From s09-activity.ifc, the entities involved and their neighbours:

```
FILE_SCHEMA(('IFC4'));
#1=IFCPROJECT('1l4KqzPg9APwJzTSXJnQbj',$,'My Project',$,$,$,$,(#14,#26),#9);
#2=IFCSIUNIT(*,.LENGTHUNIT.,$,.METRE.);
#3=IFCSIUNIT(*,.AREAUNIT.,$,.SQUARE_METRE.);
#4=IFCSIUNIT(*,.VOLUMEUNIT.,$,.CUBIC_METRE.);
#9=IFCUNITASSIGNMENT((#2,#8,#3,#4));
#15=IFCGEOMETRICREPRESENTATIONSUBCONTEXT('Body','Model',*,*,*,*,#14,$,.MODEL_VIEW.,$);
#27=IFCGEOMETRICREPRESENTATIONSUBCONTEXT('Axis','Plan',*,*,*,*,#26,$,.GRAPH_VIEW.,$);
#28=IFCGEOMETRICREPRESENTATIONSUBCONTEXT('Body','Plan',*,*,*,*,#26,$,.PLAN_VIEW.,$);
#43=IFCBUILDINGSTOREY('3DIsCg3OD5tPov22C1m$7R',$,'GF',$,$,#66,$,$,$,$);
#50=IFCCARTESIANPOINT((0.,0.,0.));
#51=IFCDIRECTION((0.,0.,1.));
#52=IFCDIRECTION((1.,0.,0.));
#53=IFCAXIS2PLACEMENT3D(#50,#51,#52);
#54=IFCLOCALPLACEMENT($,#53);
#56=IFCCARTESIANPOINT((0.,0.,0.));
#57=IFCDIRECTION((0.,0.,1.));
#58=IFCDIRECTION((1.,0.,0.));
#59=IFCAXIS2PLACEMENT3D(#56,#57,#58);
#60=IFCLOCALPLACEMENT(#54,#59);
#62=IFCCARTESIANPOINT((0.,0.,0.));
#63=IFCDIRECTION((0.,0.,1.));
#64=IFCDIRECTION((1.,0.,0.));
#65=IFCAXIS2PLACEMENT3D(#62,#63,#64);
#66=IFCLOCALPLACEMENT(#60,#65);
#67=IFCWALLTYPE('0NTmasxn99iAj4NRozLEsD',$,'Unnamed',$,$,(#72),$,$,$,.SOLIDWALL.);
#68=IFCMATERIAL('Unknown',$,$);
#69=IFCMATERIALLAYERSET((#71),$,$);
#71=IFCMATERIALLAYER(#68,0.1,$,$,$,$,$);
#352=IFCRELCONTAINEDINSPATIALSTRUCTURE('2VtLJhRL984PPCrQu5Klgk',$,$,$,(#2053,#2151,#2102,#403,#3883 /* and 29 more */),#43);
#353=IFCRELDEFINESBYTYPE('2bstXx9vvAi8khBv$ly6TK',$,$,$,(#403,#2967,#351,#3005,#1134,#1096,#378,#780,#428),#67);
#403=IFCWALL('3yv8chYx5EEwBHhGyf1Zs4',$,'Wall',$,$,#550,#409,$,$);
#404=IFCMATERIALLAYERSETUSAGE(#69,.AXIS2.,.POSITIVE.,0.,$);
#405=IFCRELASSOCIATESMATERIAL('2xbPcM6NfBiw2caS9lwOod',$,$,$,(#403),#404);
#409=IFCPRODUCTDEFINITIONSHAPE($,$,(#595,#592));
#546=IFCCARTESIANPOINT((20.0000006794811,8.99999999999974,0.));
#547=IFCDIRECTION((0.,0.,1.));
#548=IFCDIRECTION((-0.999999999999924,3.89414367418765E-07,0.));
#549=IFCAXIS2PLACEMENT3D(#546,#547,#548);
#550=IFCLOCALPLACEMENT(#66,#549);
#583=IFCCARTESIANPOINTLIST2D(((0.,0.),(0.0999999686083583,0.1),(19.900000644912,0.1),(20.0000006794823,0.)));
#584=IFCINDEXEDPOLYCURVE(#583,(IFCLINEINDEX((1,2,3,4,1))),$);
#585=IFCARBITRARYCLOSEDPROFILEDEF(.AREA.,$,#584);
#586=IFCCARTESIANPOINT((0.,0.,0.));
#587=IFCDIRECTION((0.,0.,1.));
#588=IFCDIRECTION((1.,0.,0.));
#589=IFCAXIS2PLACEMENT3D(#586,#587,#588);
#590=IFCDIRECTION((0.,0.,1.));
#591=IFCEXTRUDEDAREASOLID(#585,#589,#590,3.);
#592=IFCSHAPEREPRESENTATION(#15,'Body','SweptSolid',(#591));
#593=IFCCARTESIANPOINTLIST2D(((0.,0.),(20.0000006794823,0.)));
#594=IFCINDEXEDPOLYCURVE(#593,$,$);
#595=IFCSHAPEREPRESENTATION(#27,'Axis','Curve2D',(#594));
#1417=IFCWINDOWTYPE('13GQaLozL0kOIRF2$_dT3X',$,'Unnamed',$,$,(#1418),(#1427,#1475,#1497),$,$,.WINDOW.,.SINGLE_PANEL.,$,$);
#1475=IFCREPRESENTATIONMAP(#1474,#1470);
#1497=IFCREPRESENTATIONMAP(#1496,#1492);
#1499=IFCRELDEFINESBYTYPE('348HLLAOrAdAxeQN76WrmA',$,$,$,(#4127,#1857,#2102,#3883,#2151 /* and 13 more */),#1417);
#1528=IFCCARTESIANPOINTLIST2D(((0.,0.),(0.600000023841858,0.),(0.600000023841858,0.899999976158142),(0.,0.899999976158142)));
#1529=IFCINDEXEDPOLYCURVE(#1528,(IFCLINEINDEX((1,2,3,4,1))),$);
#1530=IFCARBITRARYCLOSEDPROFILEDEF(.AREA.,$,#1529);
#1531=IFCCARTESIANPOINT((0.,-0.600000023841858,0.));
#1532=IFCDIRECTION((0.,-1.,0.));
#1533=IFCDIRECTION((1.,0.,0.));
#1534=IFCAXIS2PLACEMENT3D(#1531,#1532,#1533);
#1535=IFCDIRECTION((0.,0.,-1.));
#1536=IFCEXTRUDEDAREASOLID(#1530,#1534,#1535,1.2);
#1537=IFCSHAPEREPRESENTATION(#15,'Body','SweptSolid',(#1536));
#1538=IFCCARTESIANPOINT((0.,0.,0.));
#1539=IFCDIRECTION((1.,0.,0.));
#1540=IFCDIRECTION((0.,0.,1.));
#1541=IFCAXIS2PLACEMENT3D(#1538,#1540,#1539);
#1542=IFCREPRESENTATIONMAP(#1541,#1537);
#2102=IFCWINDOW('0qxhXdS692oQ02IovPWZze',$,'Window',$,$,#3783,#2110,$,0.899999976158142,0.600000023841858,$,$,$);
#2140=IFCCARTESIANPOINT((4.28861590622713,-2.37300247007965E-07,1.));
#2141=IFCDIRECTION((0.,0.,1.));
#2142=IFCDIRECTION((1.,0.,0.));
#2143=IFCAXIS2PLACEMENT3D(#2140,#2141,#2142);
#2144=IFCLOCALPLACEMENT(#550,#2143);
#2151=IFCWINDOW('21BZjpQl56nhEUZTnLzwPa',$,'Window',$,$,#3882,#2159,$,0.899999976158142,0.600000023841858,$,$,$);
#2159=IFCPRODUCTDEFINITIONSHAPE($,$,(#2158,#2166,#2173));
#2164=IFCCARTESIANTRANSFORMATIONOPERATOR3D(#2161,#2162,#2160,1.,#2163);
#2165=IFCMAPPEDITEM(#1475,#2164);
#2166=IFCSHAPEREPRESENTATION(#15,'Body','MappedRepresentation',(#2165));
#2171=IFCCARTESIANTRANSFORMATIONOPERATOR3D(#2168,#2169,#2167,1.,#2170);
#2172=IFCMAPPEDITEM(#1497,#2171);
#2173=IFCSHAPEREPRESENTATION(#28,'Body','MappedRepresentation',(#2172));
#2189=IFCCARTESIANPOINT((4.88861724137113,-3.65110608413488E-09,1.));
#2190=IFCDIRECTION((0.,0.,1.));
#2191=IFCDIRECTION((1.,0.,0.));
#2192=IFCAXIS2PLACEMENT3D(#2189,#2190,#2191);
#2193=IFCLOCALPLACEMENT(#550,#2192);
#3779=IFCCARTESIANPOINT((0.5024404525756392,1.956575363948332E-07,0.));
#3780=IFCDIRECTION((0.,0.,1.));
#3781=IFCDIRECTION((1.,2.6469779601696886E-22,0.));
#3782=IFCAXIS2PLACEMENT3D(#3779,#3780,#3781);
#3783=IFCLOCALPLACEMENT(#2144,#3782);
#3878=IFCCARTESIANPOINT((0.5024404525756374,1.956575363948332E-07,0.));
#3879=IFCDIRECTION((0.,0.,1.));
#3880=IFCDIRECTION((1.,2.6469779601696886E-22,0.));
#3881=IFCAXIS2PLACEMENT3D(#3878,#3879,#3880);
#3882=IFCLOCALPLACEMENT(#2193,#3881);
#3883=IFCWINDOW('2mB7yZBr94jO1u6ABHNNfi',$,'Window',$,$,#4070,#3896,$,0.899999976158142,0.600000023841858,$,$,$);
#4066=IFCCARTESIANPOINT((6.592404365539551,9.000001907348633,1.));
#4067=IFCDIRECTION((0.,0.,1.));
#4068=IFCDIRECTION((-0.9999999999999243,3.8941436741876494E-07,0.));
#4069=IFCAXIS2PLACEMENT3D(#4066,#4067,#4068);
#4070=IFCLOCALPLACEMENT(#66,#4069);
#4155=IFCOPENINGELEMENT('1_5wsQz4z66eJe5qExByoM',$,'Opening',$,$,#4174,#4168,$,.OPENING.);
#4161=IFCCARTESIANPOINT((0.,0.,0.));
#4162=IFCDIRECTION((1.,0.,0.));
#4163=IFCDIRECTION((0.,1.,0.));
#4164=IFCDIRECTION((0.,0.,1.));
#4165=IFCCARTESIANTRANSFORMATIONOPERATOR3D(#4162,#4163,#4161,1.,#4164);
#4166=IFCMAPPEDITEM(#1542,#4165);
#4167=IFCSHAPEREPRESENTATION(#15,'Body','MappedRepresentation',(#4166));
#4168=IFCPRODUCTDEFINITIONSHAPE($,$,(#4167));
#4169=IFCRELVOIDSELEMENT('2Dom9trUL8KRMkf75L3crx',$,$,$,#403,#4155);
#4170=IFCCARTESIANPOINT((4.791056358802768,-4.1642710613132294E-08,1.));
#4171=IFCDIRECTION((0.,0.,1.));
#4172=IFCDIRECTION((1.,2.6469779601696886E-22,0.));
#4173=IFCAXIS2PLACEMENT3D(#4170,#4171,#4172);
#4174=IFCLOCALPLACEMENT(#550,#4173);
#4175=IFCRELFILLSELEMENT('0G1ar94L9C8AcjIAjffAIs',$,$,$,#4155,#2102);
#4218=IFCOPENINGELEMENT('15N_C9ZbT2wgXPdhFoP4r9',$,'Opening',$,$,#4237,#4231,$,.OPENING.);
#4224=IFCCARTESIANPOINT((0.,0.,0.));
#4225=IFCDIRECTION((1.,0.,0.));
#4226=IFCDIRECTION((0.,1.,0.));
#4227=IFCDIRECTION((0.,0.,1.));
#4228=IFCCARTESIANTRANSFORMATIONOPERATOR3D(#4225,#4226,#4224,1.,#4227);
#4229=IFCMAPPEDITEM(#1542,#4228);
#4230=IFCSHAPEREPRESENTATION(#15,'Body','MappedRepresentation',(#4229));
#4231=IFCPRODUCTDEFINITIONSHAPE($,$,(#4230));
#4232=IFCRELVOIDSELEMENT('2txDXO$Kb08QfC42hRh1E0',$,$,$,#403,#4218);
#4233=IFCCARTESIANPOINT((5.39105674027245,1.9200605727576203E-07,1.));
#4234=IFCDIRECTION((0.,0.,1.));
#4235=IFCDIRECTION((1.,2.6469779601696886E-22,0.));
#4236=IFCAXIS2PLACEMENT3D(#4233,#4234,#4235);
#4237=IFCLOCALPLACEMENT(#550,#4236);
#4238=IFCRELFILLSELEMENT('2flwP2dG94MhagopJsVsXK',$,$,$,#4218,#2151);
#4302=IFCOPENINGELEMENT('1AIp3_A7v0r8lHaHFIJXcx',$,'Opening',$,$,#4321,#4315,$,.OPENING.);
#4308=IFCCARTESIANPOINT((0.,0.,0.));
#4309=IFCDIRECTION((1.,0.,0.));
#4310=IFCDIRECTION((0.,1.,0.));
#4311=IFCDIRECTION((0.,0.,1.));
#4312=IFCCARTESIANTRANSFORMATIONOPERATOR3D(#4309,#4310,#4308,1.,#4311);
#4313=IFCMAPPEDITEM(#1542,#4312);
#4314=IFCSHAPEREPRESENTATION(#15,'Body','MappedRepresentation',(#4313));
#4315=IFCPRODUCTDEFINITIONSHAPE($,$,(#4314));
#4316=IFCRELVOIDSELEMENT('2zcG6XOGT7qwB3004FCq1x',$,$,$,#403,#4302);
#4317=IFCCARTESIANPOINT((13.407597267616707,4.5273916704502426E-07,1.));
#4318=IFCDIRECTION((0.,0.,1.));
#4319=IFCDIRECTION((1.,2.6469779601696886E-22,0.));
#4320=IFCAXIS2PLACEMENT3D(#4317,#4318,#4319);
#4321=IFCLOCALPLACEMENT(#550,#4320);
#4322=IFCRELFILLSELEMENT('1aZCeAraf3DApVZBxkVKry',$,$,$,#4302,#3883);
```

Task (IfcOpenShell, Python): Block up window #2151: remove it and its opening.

```python
import ifcopenshell
import ifcopenshell.api.feature
import ifcopenshell.api.root
import ifcopenshell.geom
import ifcopenshell.util.shape

model = ifcopenshell.open("s09-activity.ifc")
settings = ifcopenshell.geom.settings()


def volume(element):
    """Net volume in cubic metres, openings subtracted."""
    shape = ifcopenshell.geom.create_shape(settings, element)
    return ifcopenshell.util.shape.get_volume(shape.geometry)


window = model.by_guid("21BZjpQl56nhEUZTnLzwPa")
opening = window.FillsVoids[0].RelatingOpeningElement
wall = opening.VoidsElements[0].RelatingBuildingElement
before = volume(wall)

ifcopenshell.api.root.remove_product(model, product=window)
ifcopenshell.api.feature.remove_feature(model, feature=opening)

after = volume(wall)

print(f"wall volume {before:.3f} -> {after:.3f} m3")

model.write("s09-activity_v2.ifc")
```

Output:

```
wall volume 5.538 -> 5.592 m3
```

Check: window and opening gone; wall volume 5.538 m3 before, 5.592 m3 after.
